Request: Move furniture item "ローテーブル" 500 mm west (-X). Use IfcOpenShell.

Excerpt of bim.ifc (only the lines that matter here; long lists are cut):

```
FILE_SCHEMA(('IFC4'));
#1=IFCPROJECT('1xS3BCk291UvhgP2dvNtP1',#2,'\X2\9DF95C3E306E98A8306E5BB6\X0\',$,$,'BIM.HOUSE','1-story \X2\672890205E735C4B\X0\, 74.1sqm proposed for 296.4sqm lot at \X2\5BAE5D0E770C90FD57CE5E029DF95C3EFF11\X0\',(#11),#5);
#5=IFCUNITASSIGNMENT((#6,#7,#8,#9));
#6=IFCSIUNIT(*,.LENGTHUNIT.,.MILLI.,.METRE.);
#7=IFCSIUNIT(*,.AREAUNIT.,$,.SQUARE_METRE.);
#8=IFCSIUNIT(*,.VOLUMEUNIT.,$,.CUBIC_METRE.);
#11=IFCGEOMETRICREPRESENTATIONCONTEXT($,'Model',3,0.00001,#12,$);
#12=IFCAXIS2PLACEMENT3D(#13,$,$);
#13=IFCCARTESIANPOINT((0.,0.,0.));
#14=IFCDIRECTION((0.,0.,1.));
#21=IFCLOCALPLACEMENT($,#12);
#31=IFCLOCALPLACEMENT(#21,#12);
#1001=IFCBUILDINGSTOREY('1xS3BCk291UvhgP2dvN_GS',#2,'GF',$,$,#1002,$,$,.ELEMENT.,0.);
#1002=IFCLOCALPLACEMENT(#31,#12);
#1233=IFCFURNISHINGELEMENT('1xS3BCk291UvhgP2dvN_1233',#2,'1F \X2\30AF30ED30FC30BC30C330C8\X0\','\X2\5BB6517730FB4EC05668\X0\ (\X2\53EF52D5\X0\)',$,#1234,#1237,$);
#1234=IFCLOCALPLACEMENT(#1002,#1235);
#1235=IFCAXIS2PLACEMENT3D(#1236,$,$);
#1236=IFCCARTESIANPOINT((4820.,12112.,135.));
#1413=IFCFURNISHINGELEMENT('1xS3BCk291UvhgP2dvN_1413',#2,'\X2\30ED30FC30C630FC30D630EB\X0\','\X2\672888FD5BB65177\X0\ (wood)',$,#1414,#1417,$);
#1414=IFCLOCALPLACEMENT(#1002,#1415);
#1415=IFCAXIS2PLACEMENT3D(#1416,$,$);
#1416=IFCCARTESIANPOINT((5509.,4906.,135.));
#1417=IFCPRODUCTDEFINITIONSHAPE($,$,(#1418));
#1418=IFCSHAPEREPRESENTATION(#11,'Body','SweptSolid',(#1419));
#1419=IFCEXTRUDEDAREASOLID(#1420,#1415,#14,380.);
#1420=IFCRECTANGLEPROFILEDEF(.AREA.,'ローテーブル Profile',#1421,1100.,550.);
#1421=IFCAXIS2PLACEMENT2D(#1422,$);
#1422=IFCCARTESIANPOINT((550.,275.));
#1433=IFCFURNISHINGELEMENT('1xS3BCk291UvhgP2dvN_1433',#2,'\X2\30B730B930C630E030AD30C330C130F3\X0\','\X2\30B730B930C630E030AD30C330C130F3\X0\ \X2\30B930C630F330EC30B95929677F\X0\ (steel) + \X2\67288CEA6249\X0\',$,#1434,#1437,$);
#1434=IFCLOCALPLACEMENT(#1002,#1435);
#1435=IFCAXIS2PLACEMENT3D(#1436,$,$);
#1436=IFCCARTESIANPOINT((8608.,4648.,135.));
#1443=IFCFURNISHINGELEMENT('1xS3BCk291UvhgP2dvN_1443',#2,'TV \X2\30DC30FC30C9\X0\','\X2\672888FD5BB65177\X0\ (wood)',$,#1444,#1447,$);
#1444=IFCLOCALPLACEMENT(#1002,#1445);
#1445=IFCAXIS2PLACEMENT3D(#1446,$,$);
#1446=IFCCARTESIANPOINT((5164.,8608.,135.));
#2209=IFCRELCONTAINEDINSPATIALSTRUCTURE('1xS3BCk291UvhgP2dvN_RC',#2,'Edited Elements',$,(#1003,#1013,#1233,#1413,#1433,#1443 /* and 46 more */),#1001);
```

```python
import ifcopenshell
import ifcopenshell.api.geometry
import ifcopenshell.util.placement
import ifcopenshell.util.unit

model = ifcopenshell.open("bim.ifc")
unit_scale = ifcopenshell.util.unit.calculate_unit_scale(model)

item = model.by_id(1413)
matrix = ifcopenshell.util.placement.get_local_placement(item.ObjectPlacement)
matrix[0, 3] -= 0.5 / unit_scale
ifcopenshell.api.geometry.edit_object_placement(model, product=item, matrix=matrix, is_si=False)

print(ifcopenshell.util.placement.get_local_placement(item.ObjectPlacement).round(3) + 0.0)

model.write("bim_rev.ifc")
```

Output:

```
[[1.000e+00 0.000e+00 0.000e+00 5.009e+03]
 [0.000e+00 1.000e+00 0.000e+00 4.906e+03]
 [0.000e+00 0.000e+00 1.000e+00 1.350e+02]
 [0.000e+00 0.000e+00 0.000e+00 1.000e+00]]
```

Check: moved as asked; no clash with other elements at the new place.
